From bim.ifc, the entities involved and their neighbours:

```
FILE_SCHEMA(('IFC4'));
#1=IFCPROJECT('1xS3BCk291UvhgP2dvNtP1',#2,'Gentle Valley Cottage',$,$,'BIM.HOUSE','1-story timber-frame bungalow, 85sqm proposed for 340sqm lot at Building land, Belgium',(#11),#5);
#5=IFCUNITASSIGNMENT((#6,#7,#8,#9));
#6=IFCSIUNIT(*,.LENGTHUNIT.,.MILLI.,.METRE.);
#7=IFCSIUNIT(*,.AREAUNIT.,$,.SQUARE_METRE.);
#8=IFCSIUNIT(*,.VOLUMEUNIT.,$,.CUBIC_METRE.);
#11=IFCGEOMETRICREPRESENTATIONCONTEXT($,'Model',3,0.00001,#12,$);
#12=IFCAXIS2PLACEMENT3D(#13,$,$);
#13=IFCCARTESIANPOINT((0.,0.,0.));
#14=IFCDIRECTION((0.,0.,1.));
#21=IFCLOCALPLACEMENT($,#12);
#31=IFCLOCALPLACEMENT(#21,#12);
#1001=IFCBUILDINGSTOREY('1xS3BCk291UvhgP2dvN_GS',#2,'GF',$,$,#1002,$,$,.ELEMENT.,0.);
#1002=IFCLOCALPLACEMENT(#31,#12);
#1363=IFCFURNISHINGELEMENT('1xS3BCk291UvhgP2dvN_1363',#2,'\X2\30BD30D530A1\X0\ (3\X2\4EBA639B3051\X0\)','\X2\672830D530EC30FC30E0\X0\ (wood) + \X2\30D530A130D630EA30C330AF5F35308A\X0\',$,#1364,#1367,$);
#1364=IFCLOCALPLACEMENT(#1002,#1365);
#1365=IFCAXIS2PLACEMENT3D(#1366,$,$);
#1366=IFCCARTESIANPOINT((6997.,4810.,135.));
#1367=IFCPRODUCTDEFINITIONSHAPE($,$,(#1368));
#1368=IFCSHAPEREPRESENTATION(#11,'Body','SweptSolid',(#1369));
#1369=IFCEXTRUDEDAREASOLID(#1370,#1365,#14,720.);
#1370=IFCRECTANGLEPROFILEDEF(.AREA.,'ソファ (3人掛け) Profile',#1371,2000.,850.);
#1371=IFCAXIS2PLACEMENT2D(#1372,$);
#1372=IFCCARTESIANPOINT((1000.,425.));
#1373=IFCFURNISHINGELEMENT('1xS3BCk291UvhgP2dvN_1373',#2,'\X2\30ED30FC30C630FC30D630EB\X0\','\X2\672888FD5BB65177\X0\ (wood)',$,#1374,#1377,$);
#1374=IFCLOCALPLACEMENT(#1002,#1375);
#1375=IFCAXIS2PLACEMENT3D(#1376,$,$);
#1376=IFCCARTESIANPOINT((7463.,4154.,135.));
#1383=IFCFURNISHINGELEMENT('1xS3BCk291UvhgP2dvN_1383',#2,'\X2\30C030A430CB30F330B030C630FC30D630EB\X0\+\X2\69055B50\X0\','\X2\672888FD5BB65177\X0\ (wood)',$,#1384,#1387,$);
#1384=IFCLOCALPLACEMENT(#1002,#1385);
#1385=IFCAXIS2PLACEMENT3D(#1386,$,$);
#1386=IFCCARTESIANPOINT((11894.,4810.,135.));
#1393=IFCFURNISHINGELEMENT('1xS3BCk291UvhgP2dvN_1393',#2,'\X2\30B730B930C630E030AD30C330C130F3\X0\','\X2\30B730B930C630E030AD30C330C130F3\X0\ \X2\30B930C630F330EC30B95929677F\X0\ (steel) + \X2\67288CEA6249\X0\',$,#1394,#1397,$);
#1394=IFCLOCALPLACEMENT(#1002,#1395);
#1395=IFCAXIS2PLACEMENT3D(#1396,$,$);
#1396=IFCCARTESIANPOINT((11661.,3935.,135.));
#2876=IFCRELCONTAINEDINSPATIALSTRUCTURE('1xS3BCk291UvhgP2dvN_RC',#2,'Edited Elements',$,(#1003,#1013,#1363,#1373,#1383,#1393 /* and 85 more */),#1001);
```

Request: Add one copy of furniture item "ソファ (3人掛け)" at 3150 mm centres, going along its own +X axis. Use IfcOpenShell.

```python
import ifcopenshell
import ifcopenshell.api.geometry
import ifcopenshell.api.root
import ifcopenshell.util.element
import ifcopenshell.util.placement
import ifcopenshell.util.unit

model = ifcopenshell.open("bim.ifc")
unit_scale = ifcopenshell.util.unit.calculate_unit_scale(model)


def reuse_history(source, copy):
    """copy_class also copies each property set's owner history, people and application; keep the originals."""
    for rel in copy.IsDefinedBy:
        if rel.is_a("IfcRelDefinesByProperties") and (history := rel.RelatingPropertyDefinition.OwnerHistory):
            rel.RelatingPropertyDefinition.OwnerHistory = source.OwnerHistory
            ifcopenshell.util.element.remove_deep2(model, history)


source = model.by_id(1363)
base = ifcopenshell.util.placement.get_local_placement(source.ObjectPlacement)
step = base[:3, 0] * 3.15 / unit_scale

for i in range(1, 2):
    copy = ifcopenshell.api.root.copy_class(model, product=source)
    copy.Representation = ifcopenshell.util.element.copy_deep(
        model, source.Representation, exclude=["IfcGeometricRepresentationContext", "IfcRepresentationMap"]
    )
    reuse_history(source, copy)
    matrix = base.copy()
    matrix[:3, 3] += i * step
    print("added at", matrix[:3, 3].round(3) + 0.0)
    ifcopenshell.api.geometry.edit_object_placement(model, product=copy, matrix=matrix, is_si=False)

model.write("bim_edited.ifc")
```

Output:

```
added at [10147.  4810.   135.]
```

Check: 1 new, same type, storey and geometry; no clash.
